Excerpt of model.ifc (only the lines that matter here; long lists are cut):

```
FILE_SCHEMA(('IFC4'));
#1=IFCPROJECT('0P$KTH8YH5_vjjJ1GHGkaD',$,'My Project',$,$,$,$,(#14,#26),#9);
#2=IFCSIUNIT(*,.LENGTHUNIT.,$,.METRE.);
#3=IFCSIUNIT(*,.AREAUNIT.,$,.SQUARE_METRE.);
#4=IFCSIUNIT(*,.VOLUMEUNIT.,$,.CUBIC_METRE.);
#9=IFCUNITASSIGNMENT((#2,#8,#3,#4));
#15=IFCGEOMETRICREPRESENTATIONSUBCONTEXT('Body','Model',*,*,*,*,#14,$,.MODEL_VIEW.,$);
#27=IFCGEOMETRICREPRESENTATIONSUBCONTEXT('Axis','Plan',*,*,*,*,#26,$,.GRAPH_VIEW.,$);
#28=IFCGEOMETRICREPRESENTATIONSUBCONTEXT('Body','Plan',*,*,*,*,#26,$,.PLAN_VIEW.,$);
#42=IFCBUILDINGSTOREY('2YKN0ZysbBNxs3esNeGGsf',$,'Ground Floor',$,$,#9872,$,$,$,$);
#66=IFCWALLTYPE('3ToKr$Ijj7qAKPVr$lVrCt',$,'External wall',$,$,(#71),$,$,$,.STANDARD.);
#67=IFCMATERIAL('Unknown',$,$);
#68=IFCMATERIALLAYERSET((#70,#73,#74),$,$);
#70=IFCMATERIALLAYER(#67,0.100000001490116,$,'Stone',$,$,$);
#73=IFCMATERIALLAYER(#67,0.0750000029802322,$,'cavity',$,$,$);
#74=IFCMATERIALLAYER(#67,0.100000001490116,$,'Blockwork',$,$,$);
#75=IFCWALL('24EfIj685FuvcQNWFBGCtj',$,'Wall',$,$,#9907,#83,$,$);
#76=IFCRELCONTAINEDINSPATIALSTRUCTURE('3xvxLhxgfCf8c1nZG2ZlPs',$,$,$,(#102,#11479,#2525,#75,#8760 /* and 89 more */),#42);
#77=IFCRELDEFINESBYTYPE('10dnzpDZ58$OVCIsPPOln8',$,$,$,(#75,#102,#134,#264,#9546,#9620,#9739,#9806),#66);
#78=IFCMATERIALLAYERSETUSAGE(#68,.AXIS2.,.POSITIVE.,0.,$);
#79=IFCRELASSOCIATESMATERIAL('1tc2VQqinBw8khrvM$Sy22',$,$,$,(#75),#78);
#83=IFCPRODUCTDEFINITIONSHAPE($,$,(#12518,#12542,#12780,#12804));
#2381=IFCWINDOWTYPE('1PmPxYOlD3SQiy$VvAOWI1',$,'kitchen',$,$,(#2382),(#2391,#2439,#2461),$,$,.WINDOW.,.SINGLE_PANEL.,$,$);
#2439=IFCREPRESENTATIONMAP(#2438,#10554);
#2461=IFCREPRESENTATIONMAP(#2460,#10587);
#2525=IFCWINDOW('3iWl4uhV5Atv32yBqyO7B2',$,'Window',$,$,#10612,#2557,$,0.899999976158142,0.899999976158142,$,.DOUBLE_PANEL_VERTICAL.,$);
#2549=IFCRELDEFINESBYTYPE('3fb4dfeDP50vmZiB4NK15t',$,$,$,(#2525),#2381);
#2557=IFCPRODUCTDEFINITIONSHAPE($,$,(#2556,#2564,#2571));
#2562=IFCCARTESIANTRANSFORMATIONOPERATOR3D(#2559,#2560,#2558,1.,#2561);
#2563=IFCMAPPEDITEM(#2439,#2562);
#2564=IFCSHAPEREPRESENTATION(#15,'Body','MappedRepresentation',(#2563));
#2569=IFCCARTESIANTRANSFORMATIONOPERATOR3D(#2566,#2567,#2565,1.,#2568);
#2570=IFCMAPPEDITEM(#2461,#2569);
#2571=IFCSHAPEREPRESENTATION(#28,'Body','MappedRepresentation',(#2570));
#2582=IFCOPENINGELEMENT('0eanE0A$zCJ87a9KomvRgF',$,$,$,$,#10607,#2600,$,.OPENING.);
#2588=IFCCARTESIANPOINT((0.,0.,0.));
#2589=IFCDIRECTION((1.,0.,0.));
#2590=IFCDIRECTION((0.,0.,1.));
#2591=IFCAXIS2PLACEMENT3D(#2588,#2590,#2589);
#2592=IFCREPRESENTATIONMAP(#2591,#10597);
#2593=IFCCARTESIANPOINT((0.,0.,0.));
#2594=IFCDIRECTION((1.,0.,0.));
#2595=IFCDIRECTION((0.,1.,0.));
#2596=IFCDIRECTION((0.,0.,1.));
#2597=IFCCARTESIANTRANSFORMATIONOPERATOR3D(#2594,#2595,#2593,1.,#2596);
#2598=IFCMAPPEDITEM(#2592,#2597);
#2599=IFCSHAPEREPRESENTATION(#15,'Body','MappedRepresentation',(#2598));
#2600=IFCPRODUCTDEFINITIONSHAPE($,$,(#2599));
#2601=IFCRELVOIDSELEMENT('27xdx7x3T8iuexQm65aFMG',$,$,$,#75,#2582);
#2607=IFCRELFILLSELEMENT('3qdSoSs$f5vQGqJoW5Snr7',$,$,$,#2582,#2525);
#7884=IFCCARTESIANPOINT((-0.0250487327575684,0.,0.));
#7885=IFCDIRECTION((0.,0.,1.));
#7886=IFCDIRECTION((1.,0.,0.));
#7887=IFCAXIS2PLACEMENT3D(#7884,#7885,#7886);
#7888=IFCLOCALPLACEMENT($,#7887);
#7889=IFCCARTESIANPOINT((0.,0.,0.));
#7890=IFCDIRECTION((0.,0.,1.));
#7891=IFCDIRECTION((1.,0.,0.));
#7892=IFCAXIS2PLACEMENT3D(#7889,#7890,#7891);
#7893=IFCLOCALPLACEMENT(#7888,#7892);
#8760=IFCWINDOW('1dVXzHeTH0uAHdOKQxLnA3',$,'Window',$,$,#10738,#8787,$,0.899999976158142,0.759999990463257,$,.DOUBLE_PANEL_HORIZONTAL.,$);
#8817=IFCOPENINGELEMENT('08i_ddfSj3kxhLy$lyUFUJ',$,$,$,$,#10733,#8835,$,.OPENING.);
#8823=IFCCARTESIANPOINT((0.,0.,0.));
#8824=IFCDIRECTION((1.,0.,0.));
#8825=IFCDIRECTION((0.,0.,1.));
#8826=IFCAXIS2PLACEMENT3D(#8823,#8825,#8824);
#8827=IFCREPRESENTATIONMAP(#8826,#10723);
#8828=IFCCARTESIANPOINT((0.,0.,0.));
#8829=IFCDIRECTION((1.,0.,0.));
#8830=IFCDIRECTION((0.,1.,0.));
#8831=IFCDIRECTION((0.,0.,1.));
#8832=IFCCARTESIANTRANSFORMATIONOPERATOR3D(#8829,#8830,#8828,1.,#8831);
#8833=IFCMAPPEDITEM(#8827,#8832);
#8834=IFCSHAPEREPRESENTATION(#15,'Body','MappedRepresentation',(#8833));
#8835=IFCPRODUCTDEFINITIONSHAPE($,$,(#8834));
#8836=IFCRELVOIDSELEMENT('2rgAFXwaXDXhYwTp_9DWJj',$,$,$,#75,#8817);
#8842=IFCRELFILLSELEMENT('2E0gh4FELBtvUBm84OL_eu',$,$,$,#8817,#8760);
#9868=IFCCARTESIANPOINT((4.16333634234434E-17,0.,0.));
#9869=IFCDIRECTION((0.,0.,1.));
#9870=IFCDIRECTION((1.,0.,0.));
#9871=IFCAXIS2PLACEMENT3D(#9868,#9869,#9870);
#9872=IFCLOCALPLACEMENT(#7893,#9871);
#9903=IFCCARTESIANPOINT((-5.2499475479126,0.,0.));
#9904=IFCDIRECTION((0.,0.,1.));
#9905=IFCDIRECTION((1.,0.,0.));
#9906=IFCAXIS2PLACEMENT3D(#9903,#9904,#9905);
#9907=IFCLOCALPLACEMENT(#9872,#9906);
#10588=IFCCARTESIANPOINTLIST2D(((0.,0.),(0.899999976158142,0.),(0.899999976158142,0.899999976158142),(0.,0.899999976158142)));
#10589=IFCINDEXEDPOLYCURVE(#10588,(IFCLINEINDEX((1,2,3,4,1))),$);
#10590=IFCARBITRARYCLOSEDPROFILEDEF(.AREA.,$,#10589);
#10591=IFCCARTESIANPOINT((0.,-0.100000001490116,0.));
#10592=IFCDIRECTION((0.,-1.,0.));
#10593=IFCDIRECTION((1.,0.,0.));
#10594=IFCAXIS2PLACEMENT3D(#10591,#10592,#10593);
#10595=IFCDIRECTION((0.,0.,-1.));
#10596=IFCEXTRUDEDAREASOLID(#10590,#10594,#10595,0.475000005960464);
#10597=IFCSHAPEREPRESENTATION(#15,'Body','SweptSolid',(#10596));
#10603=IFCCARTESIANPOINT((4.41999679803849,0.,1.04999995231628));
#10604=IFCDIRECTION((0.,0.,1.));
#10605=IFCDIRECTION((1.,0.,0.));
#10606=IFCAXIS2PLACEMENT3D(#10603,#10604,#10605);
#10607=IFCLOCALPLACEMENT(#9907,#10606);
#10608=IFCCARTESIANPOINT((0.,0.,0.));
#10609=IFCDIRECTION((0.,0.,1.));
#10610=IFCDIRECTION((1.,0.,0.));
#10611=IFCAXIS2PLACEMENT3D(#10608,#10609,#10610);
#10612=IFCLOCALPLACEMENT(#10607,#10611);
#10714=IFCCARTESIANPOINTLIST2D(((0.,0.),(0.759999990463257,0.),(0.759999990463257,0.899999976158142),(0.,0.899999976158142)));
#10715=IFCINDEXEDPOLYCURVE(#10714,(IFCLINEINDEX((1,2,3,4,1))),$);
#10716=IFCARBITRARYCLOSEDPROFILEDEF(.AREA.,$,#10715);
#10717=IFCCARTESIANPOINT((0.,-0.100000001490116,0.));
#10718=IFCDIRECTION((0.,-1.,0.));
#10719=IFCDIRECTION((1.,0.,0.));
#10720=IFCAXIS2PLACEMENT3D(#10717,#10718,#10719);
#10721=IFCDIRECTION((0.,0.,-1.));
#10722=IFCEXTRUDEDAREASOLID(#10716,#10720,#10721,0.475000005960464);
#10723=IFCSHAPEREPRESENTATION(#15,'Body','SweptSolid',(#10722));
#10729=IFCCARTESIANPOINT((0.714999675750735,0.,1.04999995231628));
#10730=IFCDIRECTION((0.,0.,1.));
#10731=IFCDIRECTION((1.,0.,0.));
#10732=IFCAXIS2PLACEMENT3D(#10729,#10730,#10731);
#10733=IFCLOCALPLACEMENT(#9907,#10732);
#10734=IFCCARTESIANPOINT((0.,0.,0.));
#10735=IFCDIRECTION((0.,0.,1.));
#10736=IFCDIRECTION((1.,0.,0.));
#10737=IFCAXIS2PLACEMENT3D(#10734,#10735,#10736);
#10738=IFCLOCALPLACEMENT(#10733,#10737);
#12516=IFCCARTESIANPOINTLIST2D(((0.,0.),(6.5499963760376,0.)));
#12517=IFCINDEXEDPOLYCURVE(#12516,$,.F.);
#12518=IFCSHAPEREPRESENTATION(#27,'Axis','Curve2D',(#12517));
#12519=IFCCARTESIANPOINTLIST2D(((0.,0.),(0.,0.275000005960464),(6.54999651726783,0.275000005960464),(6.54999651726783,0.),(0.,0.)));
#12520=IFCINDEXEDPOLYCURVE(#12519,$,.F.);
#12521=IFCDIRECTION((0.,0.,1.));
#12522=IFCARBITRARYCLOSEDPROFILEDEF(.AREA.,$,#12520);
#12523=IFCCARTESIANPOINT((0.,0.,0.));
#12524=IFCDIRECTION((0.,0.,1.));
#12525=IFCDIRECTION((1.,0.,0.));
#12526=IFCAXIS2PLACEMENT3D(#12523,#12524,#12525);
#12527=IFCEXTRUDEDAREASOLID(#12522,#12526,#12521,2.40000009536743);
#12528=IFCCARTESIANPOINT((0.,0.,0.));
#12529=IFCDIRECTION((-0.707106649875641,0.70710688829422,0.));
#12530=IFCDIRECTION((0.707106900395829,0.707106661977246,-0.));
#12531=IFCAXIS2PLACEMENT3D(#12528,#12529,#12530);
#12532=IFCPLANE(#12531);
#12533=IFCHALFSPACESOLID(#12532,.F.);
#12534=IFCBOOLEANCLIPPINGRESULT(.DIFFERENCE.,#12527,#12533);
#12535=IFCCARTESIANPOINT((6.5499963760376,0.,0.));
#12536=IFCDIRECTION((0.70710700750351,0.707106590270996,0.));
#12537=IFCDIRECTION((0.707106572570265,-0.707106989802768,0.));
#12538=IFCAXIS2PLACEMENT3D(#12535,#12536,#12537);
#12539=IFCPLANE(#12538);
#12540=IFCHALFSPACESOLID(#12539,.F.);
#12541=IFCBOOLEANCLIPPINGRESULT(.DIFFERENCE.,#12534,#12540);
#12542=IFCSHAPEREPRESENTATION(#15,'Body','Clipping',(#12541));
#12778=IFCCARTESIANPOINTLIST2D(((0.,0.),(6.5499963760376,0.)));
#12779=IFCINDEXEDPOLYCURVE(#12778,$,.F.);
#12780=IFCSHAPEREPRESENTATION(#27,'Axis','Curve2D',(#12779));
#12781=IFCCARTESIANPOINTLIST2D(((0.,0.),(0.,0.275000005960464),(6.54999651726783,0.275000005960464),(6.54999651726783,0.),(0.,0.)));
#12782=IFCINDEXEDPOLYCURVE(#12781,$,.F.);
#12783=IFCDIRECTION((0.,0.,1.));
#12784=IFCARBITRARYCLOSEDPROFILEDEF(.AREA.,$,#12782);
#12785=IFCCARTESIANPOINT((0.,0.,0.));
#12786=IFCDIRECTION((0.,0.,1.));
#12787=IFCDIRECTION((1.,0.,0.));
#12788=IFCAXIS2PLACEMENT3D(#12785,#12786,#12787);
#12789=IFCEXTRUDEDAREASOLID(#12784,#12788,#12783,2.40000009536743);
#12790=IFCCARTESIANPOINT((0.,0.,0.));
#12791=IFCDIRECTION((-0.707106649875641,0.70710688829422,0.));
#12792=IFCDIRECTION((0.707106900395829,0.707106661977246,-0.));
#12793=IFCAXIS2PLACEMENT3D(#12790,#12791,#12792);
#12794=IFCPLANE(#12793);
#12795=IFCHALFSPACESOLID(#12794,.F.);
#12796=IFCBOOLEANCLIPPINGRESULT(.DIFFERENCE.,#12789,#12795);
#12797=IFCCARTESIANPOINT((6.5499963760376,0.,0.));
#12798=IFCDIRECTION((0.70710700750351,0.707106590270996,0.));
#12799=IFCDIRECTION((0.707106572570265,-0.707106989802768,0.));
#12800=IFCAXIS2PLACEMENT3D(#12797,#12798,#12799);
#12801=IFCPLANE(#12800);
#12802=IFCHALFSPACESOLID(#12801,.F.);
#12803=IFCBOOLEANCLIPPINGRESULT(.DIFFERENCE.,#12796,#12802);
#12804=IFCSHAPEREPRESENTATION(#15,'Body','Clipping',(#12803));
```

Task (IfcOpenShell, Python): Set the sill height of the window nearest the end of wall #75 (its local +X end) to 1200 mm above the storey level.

```python
import numpy as np
import ifcopenshell
import ifcopenshell.api.geometry
import ifcopenshell.geom
import ifcopenshell.util.element
import ifcopenshell.util.placement
import ifcopenshell.util.shape
import ifcopenshell.util.unit

model = ifcopenshell.open("model.ifc")
unit_scale = ifcopenshell.util.unit.calculate_unit_scale(model)

window = model.by_guid("3iWl4uhV5Atv32yBqyO7B2")
opening = window.FillsVoids[0].RelatingOpeningElement
storey = ifcopenshell.util.element.get_container(window, ifc_class="IfcBuildingStorey")
level = ifcopenshell.util.placement.get_local_placement(storey.ObjectPlacement)[2, 3]

# The opening's origin need not be at the sill, so measure its lowest point.
shape = ifcopenshell.geom.create_shape(ifcopenshell.geom.settings(), opening)
bottom = ifcopenshell.util.shape.get_shape_bottom_elevation(shape, shape.geometry) / unit_scale
dz = level + 1.2 / unit_scale - bottom

shift = np.array([0.0, 0.0, dz])
# The window is placed relative to its opening, so it follows when the opening moves.
matrix = ifcopenshell.util.placement.get_local_placement(opening.ObjectPlacement)
matrix[:3, 3] += shift
ifcopenshell.api.geometry.edit_object_placement(
    model, product=opening, matrix=matrix, is_si=False, should_transform_children=True
)

print(f"moved by {dz * unit_scale:+.3f} m")

model.write("model_edited.ifc")
```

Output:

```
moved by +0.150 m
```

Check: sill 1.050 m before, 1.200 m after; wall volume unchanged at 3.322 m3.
